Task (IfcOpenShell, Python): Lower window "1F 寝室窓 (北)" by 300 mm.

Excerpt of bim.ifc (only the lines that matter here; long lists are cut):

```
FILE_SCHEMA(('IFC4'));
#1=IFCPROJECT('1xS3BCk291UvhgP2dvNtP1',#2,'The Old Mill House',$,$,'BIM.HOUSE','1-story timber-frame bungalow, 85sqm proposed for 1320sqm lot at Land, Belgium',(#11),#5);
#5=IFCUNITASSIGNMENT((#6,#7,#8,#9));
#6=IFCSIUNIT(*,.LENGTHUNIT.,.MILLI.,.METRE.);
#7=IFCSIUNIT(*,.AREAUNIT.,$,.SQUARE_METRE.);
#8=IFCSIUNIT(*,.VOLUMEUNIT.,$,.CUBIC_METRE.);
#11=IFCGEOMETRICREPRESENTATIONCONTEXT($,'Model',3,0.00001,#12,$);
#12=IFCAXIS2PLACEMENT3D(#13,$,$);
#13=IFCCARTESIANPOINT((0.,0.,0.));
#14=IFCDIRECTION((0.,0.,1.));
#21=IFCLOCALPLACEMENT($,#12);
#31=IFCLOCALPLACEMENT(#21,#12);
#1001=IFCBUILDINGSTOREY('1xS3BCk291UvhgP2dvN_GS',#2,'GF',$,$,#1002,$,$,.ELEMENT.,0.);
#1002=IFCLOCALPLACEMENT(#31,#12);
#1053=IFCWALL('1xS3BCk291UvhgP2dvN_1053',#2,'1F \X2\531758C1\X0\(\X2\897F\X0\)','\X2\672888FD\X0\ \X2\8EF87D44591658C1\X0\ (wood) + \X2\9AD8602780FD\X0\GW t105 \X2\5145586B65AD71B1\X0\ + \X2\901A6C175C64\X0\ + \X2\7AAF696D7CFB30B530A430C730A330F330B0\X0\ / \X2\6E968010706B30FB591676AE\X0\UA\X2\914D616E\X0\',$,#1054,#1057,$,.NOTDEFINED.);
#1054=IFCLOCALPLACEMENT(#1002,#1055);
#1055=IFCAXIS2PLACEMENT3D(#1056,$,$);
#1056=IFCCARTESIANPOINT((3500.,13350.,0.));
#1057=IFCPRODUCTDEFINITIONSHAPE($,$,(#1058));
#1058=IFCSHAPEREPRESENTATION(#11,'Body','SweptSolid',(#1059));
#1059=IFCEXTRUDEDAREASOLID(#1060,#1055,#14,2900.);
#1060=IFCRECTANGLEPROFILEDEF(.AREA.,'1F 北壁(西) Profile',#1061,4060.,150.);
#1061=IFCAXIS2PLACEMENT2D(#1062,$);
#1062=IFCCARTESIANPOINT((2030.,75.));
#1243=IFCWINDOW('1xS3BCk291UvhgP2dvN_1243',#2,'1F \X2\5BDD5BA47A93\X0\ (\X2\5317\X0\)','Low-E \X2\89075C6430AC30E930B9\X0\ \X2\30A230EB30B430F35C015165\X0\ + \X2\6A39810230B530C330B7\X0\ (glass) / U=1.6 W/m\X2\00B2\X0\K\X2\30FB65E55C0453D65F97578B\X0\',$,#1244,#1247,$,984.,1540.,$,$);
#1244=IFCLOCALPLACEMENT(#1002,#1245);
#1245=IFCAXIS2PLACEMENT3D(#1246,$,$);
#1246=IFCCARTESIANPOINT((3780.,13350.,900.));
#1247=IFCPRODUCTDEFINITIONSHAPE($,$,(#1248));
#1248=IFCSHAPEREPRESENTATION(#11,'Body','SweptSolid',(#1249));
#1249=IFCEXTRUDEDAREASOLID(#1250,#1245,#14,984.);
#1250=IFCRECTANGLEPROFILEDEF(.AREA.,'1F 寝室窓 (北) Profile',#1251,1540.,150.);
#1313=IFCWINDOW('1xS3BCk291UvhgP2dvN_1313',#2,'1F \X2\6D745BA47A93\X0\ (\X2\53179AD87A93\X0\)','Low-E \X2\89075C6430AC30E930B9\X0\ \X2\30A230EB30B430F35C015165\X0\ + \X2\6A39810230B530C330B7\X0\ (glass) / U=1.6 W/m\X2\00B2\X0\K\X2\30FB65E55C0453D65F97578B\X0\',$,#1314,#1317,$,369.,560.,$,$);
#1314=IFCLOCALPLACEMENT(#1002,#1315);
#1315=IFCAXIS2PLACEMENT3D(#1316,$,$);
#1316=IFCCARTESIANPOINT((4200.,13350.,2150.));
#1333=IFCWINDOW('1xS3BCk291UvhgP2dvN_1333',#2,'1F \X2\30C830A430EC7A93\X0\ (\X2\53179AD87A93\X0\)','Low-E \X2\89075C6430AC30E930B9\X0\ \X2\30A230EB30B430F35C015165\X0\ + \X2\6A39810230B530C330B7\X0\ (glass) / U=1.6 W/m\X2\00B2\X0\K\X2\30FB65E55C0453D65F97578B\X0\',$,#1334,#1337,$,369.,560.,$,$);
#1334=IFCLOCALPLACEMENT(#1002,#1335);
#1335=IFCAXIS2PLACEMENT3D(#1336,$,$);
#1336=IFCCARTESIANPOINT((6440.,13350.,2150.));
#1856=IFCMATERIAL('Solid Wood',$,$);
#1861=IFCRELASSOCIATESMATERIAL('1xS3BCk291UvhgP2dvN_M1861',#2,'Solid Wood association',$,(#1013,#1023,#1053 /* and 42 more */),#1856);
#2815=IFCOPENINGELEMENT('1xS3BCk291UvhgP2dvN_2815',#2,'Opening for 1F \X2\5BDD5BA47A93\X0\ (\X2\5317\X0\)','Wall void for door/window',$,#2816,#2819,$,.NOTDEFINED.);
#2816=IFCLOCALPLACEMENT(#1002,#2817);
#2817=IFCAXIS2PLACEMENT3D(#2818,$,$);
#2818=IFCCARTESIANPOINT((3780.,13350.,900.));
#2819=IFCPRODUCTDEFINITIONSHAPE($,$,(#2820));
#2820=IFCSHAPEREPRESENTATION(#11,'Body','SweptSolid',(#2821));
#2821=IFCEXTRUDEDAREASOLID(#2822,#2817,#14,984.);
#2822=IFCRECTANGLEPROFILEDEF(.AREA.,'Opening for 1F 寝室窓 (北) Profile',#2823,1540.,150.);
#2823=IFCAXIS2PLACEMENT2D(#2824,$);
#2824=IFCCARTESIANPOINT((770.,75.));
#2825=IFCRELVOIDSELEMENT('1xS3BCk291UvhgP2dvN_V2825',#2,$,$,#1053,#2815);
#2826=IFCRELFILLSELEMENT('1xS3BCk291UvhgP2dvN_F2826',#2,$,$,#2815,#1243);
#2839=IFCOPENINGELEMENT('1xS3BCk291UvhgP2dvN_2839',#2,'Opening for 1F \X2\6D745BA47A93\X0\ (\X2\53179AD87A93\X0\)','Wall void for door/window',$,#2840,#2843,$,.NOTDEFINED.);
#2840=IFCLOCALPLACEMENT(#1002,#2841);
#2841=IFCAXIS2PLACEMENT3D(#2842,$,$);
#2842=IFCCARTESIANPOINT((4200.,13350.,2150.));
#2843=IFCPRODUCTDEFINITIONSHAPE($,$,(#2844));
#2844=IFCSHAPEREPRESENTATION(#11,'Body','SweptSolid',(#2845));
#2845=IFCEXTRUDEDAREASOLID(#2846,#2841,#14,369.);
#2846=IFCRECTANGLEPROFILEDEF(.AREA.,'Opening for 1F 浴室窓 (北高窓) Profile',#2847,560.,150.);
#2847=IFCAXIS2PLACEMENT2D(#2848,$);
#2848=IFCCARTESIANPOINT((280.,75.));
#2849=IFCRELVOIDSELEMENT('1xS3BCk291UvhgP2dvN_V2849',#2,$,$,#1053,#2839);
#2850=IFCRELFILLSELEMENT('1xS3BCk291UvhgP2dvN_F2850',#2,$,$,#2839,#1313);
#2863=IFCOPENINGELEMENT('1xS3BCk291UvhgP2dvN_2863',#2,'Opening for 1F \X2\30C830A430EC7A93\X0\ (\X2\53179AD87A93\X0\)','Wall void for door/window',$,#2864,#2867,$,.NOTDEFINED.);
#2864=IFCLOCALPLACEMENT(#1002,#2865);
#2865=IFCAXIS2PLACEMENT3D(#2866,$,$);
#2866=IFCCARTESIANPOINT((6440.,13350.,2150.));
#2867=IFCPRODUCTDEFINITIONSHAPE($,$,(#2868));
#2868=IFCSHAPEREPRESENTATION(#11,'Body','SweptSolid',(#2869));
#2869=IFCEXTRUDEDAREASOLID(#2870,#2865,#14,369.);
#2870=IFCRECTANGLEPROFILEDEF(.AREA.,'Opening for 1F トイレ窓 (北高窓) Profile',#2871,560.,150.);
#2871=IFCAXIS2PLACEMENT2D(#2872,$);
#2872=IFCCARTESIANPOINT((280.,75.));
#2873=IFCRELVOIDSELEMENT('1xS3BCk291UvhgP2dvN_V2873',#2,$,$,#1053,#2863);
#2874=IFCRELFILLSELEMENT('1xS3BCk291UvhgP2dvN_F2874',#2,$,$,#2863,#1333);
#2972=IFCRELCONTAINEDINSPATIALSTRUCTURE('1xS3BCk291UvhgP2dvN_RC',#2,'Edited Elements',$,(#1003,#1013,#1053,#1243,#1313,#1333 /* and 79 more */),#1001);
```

```python
import numpy as np
import ifcopenshell
import ifcopenshell.api.geometry
import ifcopenshell.util.placement
import ifcopenshell.util.unit

model = ifcopenshell.open("bim.ifc")
unit_scale = ifcopenshell.util.unit.calculate_unit_scale(model)

window = model.by_guid("1xS3BCk291UvhgP2dvN_1243")
opening = window.FillsVoids[0].RelatingOpeningElement
dz = -0.3 / unit_scale

shift = np.array([0.0, 0.0, dz])
# The window is not placed relative to its opening, so move both.
for product in (opening, window):
    matrix = ifcopenshell.util.placement.get_local_placement(product.ObjectPlacement)
    matrix[:3, 3] += shift
    ifcopenshell.api.geometry.edit_object_placement(model, product=product, matrix=matrix, is_si=False)

print(f"moved by {dz * unit_scale:+.3f} m")

model.write("bim_v2.ifc")
```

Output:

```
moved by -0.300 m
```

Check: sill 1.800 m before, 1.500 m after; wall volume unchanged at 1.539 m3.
